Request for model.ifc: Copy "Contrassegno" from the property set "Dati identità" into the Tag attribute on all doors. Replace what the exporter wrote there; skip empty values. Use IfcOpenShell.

First a look at what the model holds.

```python
import ifcopenshell
import ifcopenshell.util.element

model = ifcopenshell.open("model.ifc")
print(model.schema)
doors = model.by_type("IfcDoor")
print(len(doors), "doors")
for e in doors[:8]:
    source = ifcopenshell.util.element.get_pset(e, "Dati identità", "Contrassegno")
    target = e.Tag
    print(e.id(), repr(source), repr(target), sep=" | ")
```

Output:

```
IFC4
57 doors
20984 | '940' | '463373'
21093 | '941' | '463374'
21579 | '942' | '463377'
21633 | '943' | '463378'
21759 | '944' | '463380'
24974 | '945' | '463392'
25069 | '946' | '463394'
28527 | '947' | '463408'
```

```python
import ifcopenshell
import ifcopenshell.util.element

model = ifcopenshell.open("model.ifc")

count = 0
for e in model.by_type("IfcDoor"):
    value = ifcopenshell.util.element.get_pset(e, "Dati identità", "Contrassegno")
    current = e.Tag
    if not value or not value.strip() or current == value:
        continue
    e.Tag = value
    count += 1

print(count, "doors updated")

model.write("model-out.ifc")
```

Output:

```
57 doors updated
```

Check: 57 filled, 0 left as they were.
